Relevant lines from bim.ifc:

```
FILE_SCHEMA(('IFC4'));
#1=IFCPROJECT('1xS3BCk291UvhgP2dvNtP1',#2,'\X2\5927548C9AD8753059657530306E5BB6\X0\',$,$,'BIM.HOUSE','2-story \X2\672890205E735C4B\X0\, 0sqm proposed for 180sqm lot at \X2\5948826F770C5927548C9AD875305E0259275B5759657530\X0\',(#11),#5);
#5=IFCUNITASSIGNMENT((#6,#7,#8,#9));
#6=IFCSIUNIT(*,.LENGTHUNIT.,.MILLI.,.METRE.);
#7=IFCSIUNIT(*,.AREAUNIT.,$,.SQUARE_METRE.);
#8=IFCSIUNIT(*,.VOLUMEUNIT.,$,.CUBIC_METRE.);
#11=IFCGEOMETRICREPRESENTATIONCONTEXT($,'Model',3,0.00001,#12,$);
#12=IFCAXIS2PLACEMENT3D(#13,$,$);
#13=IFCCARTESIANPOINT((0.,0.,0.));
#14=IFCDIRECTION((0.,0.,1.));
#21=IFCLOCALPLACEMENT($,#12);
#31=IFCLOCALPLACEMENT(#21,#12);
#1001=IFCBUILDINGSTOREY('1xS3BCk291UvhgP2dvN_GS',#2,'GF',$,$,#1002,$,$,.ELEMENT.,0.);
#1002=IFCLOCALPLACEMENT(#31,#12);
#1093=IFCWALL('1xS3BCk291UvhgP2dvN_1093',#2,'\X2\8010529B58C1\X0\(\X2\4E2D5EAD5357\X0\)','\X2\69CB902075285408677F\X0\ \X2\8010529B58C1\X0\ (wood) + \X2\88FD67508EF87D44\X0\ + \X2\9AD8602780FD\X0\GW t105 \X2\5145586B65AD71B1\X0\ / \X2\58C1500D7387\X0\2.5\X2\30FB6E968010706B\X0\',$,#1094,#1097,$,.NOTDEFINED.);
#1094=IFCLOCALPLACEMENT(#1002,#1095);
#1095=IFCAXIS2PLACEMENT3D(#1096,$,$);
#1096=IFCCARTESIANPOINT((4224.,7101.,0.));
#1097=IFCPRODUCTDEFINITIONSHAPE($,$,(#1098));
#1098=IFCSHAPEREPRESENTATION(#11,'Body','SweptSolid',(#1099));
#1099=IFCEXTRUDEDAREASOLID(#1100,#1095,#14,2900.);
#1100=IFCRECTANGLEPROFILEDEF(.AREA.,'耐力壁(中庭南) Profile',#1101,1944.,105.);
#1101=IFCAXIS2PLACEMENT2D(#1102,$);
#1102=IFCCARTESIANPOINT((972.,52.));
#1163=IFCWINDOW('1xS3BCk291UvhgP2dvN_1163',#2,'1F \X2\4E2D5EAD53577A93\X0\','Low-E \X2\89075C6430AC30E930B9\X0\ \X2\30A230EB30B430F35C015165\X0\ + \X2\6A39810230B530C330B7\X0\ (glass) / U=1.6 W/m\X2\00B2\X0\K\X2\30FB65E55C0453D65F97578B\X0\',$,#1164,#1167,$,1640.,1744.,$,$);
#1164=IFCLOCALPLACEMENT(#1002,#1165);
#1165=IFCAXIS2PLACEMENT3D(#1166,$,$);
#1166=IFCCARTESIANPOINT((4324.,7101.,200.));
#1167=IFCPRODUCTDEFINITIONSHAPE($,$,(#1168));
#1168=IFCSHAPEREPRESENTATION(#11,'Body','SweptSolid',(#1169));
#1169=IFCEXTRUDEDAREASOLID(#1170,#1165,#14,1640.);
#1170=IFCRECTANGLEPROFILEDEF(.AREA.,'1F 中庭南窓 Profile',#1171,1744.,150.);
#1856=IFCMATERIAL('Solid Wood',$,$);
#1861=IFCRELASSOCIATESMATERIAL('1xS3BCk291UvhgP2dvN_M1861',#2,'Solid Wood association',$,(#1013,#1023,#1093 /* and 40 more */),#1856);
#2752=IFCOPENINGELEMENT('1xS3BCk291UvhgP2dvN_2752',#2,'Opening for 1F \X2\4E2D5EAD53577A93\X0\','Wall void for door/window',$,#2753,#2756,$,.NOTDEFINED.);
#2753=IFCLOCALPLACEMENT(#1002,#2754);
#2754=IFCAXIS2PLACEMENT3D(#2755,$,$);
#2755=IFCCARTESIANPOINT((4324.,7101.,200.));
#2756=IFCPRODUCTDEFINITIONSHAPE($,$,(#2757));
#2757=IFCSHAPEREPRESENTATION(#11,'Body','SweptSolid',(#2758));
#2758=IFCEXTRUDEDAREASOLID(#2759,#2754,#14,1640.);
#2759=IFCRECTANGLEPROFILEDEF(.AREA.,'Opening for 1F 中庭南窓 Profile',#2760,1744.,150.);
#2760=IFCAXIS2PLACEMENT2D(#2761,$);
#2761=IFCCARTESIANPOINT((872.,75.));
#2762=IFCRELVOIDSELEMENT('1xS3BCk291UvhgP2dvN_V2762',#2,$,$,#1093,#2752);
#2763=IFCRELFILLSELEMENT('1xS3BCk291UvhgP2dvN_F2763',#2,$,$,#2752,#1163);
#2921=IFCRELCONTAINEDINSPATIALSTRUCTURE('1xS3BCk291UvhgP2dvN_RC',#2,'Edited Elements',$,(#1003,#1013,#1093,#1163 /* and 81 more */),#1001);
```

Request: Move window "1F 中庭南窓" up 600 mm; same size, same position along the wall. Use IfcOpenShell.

```python
import numpy as np
import ifcopenshell
import ifcopenshell.api.geometry
import ifcopenshell.util.placement
import ifcopenshell.util.unit

model = ifcopenshell.open("bim.ifc")
unit_scale = ifcopenshell.util.unit.calculate_unit_scale(model)

window = model.by_guid("1xS3BCk291UvhgP2dvN_1163")
opening = window.FillsVoids[0].RelatingOpeningElement
dz = 0.6 / unit_scale

shift = np.array([0.0, 0.0, dz])
# The window is not placed relative to its opening, so move both.
for product in (opening, window):
    matrix = ifcopenshell.util.placement.get_local_placement(product.ObjectPlacement)
    matrix[:3, 3] += shift
    ifcopenshell.api.geometry.edit_object_placement(model, product=product, matrix=matrix, is_si=False)

print(f"moved by {dz * unit_scale:+.3f} m")

model.write("bim-out.ifc")
```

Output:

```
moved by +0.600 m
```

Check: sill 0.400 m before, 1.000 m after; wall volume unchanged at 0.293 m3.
